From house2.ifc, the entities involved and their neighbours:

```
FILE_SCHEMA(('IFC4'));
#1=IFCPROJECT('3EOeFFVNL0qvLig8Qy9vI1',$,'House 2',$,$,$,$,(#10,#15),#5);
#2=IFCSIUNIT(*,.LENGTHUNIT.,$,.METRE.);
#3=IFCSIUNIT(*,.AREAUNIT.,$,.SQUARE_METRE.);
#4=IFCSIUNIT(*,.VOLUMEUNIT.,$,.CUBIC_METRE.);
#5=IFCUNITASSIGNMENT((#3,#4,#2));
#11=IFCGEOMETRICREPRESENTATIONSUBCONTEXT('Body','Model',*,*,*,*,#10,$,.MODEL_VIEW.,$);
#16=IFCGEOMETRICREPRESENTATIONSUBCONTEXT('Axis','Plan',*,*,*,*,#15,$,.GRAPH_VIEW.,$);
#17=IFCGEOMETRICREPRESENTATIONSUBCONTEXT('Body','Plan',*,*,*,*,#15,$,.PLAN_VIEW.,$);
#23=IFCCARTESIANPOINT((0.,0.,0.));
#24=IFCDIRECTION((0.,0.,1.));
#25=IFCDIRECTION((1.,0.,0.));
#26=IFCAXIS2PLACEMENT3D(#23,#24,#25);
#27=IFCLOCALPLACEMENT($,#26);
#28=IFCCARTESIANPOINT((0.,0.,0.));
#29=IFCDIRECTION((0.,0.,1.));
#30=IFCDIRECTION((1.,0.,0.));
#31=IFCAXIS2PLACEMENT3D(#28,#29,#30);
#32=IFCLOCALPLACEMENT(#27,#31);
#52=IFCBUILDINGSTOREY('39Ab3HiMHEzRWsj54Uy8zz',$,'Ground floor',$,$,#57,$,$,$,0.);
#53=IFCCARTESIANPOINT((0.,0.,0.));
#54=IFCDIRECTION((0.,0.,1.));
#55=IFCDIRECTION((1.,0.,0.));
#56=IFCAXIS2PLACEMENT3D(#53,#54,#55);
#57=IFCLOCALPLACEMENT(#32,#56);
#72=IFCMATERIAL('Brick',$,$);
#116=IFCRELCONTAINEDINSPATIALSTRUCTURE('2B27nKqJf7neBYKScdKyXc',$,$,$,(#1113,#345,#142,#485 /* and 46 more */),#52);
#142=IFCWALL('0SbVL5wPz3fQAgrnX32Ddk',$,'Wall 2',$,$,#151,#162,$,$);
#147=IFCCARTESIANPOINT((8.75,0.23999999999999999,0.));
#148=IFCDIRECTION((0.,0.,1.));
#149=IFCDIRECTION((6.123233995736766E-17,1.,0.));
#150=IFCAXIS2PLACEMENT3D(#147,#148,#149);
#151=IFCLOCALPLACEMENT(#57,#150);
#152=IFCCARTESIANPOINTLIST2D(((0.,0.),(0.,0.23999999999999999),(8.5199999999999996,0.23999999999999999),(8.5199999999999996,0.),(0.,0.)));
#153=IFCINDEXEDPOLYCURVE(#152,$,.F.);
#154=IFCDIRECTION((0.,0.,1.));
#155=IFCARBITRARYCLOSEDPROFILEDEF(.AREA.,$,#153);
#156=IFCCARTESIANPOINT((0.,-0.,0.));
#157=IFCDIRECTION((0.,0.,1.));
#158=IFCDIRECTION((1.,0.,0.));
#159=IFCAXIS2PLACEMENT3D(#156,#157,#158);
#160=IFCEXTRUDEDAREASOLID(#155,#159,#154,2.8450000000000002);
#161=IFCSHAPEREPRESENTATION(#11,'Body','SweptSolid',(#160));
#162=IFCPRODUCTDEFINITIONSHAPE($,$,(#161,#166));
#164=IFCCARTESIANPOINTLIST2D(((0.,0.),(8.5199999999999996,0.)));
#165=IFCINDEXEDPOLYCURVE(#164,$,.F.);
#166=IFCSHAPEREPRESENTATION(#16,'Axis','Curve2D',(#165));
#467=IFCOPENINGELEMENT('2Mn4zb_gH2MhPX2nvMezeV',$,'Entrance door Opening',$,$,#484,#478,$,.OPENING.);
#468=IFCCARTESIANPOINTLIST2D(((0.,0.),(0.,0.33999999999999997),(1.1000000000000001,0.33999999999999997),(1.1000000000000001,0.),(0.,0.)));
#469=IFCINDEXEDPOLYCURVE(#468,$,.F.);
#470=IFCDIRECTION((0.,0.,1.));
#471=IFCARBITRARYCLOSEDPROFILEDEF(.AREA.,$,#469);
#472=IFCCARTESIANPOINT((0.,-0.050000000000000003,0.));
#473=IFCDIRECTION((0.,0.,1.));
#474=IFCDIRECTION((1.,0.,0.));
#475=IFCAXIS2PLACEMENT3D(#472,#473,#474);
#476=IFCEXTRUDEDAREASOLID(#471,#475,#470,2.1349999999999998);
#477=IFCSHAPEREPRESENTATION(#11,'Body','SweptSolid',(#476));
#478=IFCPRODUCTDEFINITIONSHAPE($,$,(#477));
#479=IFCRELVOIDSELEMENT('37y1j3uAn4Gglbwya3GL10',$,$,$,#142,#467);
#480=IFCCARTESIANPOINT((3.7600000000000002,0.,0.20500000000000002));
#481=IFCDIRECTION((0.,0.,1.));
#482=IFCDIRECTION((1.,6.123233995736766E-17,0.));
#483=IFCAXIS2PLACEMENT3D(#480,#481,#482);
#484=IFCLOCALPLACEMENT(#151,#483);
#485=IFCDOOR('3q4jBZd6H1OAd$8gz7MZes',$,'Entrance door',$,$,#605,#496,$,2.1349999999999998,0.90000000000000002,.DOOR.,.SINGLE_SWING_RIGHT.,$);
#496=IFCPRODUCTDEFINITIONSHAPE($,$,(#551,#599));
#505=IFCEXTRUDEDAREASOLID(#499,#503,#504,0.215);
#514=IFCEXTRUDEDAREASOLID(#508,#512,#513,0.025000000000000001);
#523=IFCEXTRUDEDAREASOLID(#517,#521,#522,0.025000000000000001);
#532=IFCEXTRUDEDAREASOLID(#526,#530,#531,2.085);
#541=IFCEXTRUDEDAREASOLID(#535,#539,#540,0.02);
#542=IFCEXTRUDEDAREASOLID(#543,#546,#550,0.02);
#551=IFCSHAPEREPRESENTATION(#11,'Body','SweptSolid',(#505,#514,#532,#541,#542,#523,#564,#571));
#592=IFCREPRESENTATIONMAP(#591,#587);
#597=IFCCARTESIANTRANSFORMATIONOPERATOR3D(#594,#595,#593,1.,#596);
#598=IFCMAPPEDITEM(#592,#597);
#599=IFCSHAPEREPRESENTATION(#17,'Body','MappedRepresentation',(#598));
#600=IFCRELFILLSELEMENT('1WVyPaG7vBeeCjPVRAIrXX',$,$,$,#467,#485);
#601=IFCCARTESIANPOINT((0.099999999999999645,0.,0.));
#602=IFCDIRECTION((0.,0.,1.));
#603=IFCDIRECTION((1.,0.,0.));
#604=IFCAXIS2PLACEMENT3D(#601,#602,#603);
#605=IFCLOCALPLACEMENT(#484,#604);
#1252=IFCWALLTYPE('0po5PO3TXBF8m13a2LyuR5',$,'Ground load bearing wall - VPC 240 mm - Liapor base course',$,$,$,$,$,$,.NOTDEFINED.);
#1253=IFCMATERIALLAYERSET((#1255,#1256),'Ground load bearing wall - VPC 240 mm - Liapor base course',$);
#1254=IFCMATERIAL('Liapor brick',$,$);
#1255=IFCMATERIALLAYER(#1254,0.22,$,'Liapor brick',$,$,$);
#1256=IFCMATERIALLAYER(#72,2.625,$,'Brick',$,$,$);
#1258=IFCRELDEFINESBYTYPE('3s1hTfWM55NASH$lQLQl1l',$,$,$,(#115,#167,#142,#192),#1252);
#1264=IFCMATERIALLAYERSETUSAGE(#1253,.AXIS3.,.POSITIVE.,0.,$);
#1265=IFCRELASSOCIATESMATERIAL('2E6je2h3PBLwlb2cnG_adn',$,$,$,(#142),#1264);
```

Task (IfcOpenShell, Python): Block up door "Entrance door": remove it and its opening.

```python
import ifcopenshell
import ifcopenshell.api.feature
import ifcopenshell.api.root
import ifcopenshell.geom
import ifcopenshell.util.shape

model = ifcopenshell.open("house2.ifc")
settings = ifcopenshell.geom.settings()


def volume(element):
    """Net volume in cubic metres, openings subtracted."""
    shape = ifcopenshell.geom.create_shape(settings, element)
    return ifcopenshell.util.shape.get_volume(shape.geometry)


door = model.by_guid("3q4jBZd6H1OAd$8gz7MZes")
opening = door.FillsVoids[0].RelatingOpeningElement
wall = opening.VoidsElements[0].RelatingBuildingElement
before = volume(wall)

ifcopenshell.api.root.remove_product(model, product=door)
ifcopenshell.api.feature.remove_feature(model, feature=opening)

after = volume(wall)

print(f"wall volume {before:.3f} -> {after:.3f} m3")

model.write("house2_v2.ifc")
```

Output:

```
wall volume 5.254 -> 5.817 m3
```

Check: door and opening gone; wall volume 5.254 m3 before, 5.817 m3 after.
